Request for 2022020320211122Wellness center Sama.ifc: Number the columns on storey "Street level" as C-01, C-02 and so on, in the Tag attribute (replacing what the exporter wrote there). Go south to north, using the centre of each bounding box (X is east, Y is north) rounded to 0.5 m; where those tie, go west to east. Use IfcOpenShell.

First a look at what the model holds.

```python
import ifcopenshell
import ifcopenshell.util.element
import ifcopenshell.util.placement

model = ifcopenshell.open("2022020320211122Wellness center Sama.ifc")
print(model.schema)
storey = next(s for s in model.by_type("IfcBuildingStorey") if s.Name == "Street level")
columns = [e for e in ifcopenshell.util.element.get_decomposition(storey) if e.is_a("IfcColumn")]
for e in sorted(columns, key=lambda e: e.id()):
    origin = ifcopenshell.util.placement.get_local_placement(e.ObjectPlacement)[:3, 3]
    print(e.id(), e.Tag, e.Name, origin.round(2) + 0.0, sep=" | ")
```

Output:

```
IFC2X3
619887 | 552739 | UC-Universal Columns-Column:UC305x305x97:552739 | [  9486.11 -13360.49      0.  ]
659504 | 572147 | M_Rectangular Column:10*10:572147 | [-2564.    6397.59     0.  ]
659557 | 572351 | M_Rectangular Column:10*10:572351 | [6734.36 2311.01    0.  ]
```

```python
import ifcopenshell
import ifcopenshell.geom
import ifcopenshell.util.element
import ifcopenshell.util.shape

model = ifcopenshell.open("2022020320211122Wellness center Sama.ifc")
settings = ifcopenshell.geom.settings()
settings.set("use-world-coords", True)


def centre(element):
    shape = ifcopenshell.geom.create_shape(settings, element)
    return ifcopenshell.util.shape.get_bbox_centroid(shape.geometry)


storey = next(s for s in model.by_type("IfcBuildingStorey") if s.Name == "Street level")
columns = [e for e in ifcopenshell.util.element.get_decomposition(storey) if e.is_a("IfcColumn")]

# Insertion points can sit at a corner or the storey origin, so sort by the geometry (in metres).
centres = {e: centre(e) for e in columns}
columns.sort(key=lambda e: (round(centres[e][1] / 0.5), centres[e][0]))

for i, e in enumerate(columns, start=1):
    number = f"C-{i:02d}"
    e.Tag = number
    print(e.id(), number)

model.write("2022020320211122Wellness center Sama_edited.ifc")
```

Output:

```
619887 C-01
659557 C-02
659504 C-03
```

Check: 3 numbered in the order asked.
